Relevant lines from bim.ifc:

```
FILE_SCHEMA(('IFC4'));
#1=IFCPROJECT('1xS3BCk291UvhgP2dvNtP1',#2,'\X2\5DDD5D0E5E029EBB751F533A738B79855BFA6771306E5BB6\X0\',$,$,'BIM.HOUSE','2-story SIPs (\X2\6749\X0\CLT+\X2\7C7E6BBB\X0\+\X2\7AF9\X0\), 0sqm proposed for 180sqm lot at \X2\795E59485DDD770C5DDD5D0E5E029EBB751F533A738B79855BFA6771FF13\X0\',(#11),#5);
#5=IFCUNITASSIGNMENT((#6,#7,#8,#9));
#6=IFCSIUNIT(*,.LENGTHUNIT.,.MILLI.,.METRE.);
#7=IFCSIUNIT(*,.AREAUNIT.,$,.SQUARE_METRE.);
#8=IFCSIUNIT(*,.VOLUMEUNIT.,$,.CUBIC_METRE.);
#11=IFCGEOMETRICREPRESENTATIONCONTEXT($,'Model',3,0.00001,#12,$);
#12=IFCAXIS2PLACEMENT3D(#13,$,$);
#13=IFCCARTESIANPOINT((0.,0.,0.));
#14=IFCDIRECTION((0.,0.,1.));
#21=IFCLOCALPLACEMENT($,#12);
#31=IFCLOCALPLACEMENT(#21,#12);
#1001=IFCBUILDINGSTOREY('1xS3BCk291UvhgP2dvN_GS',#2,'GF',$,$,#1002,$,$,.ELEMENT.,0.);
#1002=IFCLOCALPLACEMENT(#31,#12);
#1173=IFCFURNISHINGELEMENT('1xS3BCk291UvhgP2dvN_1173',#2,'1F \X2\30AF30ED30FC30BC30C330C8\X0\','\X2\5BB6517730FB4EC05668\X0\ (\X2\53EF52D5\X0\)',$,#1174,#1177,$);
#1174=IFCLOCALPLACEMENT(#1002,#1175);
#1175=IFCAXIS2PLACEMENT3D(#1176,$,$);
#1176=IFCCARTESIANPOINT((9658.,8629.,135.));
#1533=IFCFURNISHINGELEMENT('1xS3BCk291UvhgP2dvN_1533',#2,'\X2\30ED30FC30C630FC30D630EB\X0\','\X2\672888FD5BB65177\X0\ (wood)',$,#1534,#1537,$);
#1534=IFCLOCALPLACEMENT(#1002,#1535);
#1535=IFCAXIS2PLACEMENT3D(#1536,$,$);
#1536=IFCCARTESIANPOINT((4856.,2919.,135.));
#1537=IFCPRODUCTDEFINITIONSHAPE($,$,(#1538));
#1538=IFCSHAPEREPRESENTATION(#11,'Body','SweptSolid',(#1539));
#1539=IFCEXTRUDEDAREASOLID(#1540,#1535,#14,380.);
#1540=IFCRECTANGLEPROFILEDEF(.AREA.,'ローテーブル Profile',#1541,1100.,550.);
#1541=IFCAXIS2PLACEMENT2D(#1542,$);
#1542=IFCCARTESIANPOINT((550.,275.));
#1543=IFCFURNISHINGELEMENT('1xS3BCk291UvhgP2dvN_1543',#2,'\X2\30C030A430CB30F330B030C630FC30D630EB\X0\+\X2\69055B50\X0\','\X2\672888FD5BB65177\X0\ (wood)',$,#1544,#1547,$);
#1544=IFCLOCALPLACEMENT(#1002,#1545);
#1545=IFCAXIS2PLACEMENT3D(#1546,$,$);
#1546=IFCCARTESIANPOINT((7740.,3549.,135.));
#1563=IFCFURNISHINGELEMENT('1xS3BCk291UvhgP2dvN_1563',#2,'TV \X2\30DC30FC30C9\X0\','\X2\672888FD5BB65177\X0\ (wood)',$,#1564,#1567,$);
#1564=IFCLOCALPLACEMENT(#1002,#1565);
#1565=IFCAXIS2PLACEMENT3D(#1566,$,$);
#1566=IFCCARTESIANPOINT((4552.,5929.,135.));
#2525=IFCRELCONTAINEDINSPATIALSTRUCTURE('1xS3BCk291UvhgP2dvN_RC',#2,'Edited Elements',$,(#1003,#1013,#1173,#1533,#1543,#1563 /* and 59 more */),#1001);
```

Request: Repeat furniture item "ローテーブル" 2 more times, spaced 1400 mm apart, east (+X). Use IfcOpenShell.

```python
import numpy as np
import ifcopenshell
import ifcopenshell.api.geometry
import ifcopenshell.api.root
import ifcopenshell.util.element
import ifcopenshell.util.placement
import ifcopenshell.util.unit

model = ifcopenshell.open("bim.ifc")
unit_scale = ifcopenshell.util.unit.calculate_unit_scale(model)


def reuse_history(source, copy):
    """copy_class also copies each property set's owner history, people and application; keep the originals."""
    for rel in copy.IsDefinedBy:
        if rel.is_a("IfcRelDefinesByProperties") and (history := rel.RelatingPropertyDefinition.OwnerHistory):
            rel.RelatingPropertyDefinition.OwnerHistory = source.OwnerHistory
            ifcopenshell.util.element.remove_deep2(model, history)


source = model.by_guid("1xS3BCk291UvhgP2dvN_1533")
base = ifcopenshell.util.placement.get_local_placement(source.ObjectPlacement)
step = np.array([1.0, 0.0, 0.0]) * 1.4 / unit_scale

for i in range(1, 3):
    copy = ifcopenshell.api.root.copy_class(model, product=source)
    copy.Representation = ifcopenshell.util.element.copy_deep(
        model, source.Representation, exclude=["IfcGeometricRepresentationContext", "IfcRepresentationMap"]
    )
    reuse_history(source, copy)
    matrix = base.copy()
    matrix[:3, 3] += i * step
    print("added at", matrix[:3, 3].round(3) + 0.0)
    ifcopenshell.api.geometry.edit_object_placement(model, product=copy, matrix=matrix, is_si=False)

model.write("bim-out.ifc")
```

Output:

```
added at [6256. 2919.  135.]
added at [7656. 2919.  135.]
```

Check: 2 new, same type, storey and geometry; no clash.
